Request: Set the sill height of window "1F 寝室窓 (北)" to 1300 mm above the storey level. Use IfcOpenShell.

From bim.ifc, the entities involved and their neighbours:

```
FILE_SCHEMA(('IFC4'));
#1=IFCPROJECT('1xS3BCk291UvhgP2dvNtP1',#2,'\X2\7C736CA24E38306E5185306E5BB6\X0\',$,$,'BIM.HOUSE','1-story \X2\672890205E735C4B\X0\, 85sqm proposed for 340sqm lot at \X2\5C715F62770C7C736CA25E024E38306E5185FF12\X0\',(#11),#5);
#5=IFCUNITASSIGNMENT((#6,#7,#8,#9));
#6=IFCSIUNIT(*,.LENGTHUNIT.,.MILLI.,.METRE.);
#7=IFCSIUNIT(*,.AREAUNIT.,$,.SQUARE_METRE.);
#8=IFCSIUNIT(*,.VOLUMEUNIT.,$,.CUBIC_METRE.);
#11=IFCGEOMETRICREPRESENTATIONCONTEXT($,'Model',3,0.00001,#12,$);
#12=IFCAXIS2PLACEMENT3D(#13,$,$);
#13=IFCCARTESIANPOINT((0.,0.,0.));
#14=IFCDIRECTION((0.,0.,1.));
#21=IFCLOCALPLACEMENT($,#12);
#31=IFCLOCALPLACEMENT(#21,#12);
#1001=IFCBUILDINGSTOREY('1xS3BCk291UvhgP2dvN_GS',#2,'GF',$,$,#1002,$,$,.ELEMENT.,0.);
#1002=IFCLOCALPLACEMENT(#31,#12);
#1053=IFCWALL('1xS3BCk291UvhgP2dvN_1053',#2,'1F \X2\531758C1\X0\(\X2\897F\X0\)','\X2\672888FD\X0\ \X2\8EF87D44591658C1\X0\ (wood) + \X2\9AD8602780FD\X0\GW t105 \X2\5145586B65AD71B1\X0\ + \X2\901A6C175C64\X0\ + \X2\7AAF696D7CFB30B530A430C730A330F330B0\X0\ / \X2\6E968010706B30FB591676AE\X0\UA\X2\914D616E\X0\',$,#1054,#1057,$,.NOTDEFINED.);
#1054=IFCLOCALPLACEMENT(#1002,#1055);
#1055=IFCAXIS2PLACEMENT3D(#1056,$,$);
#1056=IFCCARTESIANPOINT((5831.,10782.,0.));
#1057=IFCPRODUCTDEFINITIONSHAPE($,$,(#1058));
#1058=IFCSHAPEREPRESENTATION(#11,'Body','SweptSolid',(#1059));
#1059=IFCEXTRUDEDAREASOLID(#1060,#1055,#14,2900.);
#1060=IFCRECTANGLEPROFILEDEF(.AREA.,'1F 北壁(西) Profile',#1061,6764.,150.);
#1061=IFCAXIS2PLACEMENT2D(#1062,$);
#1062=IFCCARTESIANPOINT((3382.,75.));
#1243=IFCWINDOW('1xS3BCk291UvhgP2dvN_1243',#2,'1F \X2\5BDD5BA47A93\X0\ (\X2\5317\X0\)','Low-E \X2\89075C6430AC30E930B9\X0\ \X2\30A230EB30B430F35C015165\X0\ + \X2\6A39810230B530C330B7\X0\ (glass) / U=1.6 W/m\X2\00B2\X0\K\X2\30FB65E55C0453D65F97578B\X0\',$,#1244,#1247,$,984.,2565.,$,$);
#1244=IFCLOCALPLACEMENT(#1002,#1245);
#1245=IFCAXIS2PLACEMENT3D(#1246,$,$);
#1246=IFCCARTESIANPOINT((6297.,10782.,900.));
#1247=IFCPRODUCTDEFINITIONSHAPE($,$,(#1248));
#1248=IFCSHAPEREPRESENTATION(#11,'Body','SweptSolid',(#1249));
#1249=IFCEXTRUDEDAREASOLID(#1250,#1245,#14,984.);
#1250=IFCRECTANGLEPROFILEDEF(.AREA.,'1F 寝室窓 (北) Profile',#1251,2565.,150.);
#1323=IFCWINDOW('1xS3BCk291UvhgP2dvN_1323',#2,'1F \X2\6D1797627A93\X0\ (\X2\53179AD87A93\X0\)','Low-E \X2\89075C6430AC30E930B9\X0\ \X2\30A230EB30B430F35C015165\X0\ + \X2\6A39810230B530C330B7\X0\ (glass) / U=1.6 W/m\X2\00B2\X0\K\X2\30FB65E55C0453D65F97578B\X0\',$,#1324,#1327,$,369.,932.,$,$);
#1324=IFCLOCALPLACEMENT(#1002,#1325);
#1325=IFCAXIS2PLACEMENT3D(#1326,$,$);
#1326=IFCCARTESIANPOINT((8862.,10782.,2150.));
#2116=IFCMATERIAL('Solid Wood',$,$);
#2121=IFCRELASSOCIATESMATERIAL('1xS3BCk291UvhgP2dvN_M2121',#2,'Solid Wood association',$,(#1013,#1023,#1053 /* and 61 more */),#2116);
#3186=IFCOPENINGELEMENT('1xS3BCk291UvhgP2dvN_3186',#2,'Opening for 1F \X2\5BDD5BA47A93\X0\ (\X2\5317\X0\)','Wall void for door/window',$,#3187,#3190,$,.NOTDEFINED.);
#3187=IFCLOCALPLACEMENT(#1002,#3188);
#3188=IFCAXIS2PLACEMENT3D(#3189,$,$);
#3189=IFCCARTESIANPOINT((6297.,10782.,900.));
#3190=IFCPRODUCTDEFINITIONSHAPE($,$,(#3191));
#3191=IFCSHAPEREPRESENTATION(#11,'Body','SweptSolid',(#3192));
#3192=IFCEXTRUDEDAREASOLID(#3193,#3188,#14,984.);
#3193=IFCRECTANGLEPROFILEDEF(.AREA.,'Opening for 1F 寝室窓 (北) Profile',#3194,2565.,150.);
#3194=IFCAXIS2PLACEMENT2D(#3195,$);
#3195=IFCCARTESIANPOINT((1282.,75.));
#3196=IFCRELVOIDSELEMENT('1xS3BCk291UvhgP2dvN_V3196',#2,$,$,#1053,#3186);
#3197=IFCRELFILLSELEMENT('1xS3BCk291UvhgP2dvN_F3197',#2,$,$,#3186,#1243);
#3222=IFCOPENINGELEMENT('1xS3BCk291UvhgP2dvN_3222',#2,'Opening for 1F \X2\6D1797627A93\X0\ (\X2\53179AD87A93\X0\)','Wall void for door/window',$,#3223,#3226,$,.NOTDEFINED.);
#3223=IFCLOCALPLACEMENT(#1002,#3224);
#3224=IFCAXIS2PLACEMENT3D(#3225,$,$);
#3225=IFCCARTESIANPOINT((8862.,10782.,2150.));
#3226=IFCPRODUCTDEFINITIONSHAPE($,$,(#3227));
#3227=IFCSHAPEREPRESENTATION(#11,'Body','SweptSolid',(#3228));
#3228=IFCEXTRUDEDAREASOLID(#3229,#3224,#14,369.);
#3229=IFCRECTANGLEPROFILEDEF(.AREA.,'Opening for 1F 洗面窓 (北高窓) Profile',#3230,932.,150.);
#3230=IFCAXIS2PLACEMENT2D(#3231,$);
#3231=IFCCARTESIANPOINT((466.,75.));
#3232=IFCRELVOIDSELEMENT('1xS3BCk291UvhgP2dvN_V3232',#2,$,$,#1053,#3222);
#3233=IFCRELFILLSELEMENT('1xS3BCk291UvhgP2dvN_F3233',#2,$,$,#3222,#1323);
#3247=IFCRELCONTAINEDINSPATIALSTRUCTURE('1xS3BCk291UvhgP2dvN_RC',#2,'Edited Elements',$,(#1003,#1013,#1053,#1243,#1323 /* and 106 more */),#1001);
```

```python
import numpy as np
import ifcopenshell
import ifcopenshell.api.geometry
import ifcopenshell.geom
import ifcopenshell.util.element
import ifcopenshell.util.placement
import ifcopenshell.util.shape
import ifcopenshell.util.unit

model = ifcopenshell.open("bim.ifc")
unit_scale = ifcopenshell.util.unit.calculate_unit_scale(model)

window = model.by_guid("1xS3BCk291UvhgP2dvN_1243")
opening = window.FillsVoids[0].RelatingOpeningElement
storey = ifcopenshell.util.element.get_container(window, ifc_class="IfcBuildingStorey")
level = ifcopenshell.util.placement.get_local_placement(storey.ObjectPlacement)[2, 3]

# The opening's origin need not be at the sill, so measure its lowest point.
shape = ifcopenshell.geom.create_shape(ifcopenshell.geom.settings(), opening)
bottom = ifcopenshell.util.shape.get_shape_bottom_elevation(shape, shape.geometry) / unit_scale
dz = level + 1.3 / unit_scale - bottom

shift = np.array([0.0, 0.0, dz])
# The window is not placed relative to its opening, so move both.
for product in (opening, window):
    matrix = ifcopenshell.util.placement.get_local_placement(product.ObjectPlacement)
    matrix[:3, 3] += shift
    ifcopenshell.api.geometry.edit_object_placement(model, product=product, matrix=matrix, is_si=False)

print(f"moved by {dz * unit_scale:+.3f} m")

model.write("bim_rev.ifc")
```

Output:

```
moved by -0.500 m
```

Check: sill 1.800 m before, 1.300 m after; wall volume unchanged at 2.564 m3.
